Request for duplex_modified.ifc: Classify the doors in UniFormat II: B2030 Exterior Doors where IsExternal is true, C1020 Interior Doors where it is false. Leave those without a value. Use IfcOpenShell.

First a look at what the model holds.

```python
import ifcopenshell
import ifcopenshell.util.element

model = ifcopenshell.open("duplex_modified.ifc")
print(model.schema)
print("classifications:", [c.Name for c in model.by_type("IfcClassification")])
values = [ifcopenshell.util.element.get_pset(e, "Pset_DoorCommon", "IsExternal") for e in model.by_type("IfcDoor")]
for value in (True, False, None):
    print("IsExternal", value, values.count(value))
```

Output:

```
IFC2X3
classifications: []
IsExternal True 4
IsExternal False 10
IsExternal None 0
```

```python
import ifcopenshell
import ifcopenshell.api.classification
import ifcopenshell.util.element

model = ifcopenshell.open("duplex_modified.ifc")

# IFC2X3 requires Source and Edition and has no link from the project to the system.
system = model.create_entity("IfcClassification", Source="ASTM", Edition="E1557", Name="UniFormat II")

doors = model.by_type("IfcDoor")
external = {e: ifcopenshell.util.element.get_pset(e, "Pset_DoorCommon", "IsExternal") for e in doors}
for flag, code, name in ((True, "B2030", "Exterior Doors"), (False, "C1020", "Interior Doors")):
    products = [e for e in doors if external[e] is flag]
    ifcopenshell.api.classification.add_reference(
        model, products=products, classification=system, identification=code, name=name
    )
    print(code, len(products))

model.write("duplex_modified_edited.ifc")
```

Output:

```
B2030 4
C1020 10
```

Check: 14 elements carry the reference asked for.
